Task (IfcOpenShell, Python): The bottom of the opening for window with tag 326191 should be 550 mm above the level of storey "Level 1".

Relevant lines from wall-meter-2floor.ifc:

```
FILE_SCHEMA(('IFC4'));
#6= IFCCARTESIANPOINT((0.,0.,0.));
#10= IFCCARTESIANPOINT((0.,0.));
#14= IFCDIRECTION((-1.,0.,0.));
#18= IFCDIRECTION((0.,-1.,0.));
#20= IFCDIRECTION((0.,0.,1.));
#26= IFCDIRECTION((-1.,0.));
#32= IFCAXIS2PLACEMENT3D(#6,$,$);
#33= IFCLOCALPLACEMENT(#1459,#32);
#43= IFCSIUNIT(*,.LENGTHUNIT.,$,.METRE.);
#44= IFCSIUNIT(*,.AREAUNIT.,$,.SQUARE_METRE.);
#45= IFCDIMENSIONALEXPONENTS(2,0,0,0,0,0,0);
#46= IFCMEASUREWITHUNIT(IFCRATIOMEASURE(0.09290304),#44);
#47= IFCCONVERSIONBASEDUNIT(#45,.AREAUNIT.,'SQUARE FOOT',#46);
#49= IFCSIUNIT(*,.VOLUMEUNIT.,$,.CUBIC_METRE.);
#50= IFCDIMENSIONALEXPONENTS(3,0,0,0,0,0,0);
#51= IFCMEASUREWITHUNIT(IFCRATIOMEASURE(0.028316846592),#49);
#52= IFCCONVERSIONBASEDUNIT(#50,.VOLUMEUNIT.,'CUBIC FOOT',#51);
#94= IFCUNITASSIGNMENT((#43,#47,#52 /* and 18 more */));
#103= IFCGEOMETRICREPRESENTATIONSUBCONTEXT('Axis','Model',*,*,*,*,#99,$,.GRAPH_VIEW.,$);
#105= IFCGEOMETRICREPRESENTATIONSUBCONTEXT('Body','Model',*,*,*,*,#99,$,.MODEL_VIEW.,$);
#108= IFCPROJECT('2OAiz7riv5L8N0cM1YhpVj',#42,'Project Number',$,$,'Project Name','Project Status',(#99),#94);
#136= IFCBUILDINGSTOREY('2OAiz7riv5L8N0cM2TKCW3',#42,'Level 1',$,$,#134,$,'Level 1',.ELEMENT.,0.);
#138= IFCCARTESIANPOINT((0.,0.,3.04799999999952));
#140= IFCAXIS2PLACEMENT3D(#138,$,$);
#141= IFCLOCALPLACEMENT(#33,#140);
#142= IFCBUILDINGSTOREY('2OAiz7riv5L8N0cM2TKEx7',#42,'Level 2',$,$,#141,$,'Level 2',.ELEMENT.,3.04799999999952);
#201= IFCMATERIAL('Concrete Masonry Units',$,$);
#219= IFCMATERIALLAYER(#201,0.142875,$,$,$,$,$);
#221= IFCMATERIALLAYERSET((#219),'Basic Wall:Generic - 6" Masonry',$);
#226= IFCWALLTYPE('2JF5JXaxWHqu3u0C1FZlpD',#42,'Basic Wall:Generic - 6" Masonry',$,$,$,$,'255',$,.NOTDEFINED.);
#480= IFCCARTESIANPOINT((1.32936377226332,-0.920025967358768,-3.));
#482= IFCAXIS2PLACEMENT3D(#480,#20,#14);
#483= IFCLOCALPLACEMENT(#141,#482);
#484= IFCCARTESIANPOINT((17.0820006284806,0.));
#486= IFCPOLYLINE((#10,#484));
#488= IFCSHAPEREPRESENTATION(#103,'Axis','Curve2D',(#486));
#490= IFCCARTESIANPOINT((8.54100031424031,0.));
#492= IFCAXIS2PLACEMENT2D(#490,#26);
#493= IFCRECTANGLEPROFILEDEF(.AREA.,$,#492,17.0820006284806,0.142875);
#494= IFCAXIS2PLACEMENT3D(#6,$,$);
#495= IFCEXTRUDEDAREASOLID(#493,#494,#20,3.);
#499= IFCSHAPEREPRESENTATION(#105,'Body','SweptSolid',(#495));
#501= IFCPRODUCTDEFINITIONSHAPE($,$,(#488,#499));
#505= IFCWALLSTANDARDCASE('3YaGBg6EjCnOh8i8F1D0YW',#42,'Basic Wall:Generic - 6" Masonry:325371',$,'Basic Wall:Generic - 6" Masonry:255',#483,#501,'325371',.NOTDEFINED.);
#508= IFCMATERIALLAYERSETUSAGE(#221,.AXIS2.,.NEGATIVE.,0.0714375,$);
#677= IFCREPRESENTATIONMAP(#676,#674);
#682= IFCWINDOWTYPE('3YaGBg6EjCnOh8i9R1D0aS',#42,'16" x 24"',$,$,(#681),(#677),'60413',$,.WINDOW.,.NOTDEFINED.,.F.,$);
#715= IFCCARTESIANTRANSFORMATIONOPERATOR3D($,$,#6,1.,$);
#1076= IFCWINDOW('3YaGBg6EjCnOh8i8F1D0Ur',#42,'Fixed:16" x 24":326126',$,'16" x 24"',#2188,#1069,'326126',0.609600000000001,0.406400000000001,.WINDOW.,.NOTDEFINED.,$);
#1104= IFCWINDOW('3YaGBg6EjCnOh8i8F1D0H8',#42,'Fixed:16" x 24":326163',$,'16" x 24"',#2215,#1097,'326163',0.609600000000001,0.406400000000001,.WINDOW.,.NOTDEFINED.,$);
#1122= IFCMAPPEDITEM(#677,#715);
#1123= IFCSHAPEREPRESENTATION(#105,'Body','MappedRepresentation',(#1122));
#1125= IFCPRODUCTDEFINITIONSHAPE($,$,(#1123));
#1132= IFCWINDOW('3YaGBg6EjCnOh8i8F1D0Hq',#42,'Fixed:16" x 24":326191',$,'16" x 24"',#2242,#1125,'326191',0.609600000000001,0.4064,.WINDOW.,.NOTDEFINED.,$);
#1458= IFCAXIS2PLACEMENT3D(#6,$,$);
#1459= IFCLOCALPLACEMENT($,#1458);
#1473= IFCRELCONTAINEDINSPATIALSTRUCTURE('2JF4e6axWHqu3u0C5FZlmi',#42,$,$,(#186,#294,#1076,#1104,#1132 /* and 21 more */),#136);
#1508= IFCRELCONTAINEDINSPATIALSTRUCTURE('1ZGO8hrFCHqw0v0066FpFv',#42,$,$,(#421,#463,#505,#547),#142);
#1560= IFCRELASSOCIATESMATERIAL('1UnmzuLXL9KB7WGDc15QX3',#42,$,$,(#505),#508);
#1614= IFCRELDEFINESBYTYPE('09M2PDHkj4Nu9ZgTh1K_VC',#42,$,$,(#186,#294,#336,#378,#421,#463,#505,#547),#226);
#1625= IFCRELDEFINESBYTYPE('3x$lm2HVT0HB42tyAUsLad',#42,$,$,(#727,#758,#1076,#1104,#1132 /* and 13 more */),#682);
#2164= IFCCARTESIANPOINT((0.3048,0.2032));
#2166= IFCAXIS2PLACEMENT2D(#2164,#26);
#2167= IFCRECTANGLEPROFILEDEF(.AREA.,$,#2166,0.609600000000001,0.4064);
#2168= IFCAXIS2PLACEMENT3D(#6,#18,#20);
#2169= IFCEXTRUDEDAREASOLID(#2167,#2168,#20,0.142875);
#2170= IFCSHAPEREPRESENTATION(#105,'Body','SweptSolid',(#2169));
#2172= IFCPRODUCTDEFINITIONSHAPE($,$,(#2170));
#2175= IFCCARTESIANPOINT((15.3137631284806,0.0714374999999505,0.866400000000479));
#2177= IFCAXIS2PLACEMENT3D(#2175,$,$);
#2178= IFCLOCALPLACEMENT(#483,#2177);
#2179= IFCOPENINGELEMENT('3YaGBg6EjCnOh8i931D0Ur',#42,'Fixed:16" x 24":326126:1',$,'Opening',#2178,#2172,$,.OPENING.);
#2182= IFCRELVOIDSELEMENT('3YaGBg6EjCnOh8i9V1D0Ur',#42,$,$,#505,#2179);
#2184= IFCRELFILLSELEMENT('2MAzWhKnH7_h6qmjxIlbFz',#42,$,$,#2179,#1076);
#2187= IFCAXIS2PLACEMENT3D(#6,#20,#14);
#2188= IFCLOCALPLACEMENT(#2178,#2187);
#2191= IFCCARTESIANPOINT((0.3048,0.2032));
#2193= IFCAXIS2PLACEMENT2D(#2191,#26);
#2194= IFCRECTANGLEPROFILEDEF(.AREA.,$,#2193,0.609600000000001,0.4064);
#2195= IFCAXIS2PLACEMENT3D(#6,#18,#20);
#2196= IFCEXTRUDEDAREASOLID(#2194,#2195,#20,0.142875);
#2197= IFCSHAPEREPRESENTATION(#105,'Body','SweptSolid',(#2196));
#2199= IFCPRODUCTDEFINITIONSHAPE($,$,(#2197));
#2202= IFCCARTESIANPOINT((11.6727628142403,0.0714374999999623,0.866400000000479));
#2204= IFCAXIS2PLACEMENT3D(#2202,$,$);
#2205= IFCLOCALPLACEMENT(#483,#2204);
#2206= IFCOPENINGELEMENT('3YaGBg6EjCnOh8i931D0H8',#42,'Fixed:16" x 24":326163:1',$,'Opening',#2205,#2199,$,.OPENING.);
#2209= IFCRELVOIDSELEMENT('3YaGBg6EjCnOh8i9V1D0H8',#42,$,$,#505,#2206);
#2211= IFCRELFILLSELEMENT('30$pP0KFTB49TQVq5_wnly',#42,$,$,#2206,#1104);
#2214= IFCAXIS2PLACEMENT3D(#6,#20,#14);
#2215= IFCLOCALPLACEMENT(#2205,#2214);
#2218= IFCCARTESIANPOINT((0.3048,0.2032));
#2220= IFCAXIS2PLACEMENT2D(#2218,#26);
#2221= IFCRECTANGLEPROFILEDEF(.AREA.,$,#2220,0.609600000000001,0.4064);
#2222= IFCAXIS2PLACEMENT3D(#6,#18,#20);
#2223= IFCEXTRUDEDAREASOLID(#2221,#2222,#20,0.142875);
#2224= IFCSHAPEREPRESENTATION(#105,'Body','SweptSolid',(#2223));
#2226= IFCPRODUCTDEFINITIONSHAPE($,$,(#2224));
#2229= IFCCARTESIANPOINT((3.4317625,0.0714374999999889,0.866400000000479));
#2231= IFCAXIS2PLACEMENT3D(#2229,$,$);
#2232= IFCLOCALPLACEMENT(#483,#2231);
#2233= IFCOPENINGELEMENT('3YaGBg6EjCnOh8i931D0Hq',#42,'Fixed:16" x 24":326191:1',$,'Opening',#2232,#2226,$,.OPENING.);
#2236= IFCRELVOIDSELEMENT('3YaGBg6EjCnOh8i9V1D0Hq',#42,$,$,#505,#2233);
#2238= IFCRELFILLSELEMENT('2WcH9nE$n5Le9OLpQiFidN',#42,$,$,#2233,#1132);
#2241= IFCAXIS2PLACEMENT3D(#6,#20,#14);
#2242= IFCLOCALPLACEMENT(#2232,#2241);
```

```python
import numpy as np
import ifcopenshell
import ifcopenshell.api.geometry
import ifcopenshell.geom
import ifcopenshell.util.element
import ifcopenshell.util.placement
import ifcopenshell.util.shape
import ifcopenshell.util.unit

model = ifcopenshell.open("wall-meter-2floor.ifc")
unit_scale = ifcopenshell.util.unit.calculate_unit_scale(model)

window = model.by_guid("3YaGBg6EjCnOh8i8F1D0Hq")
opening = window.FillsVoids[0].RelatingOpeningElement
storey = ifcopenshell.util.element.get_container(window, ifc_class="IfcBuildingStorey")
level = ifcopenshell.util.placement.get_local_placement(storey.ObjectPlacement)[2, 3]

# The opening's origin need not be at the sill, so measure its lowest point.
shape = ifcopenshell.geom.create_shape(ifcopenshell.geom.settings(), opening)
bottom = ifcopenshell.util.shape.get_shape_bottom_elevation(shape, shape.geometry) / unit_scale
dz = level + 0.55 / unit_scale - bottom

shift = np.array([0.0, 0.0, dz])
# The window is placed relative to its opening, so it follows when the opening moves.
matrix = ifcopenshell.util.placement.get_local_placement(opening.ObjectPlacement)
matrix[:3, 3] += shift
ifcopenshell.api.geometry.edit_object_placement(
    model, product=opening, matrix=matrix, is_si=False, should_transform_children=True
)

print(f"moved by {dz * unit_scale:+.3f} m")

model.write("wall-meter-2floor_v2.ifc")
```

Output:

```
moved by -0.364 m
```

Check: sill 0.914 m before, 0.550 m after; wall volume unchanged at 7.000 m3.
